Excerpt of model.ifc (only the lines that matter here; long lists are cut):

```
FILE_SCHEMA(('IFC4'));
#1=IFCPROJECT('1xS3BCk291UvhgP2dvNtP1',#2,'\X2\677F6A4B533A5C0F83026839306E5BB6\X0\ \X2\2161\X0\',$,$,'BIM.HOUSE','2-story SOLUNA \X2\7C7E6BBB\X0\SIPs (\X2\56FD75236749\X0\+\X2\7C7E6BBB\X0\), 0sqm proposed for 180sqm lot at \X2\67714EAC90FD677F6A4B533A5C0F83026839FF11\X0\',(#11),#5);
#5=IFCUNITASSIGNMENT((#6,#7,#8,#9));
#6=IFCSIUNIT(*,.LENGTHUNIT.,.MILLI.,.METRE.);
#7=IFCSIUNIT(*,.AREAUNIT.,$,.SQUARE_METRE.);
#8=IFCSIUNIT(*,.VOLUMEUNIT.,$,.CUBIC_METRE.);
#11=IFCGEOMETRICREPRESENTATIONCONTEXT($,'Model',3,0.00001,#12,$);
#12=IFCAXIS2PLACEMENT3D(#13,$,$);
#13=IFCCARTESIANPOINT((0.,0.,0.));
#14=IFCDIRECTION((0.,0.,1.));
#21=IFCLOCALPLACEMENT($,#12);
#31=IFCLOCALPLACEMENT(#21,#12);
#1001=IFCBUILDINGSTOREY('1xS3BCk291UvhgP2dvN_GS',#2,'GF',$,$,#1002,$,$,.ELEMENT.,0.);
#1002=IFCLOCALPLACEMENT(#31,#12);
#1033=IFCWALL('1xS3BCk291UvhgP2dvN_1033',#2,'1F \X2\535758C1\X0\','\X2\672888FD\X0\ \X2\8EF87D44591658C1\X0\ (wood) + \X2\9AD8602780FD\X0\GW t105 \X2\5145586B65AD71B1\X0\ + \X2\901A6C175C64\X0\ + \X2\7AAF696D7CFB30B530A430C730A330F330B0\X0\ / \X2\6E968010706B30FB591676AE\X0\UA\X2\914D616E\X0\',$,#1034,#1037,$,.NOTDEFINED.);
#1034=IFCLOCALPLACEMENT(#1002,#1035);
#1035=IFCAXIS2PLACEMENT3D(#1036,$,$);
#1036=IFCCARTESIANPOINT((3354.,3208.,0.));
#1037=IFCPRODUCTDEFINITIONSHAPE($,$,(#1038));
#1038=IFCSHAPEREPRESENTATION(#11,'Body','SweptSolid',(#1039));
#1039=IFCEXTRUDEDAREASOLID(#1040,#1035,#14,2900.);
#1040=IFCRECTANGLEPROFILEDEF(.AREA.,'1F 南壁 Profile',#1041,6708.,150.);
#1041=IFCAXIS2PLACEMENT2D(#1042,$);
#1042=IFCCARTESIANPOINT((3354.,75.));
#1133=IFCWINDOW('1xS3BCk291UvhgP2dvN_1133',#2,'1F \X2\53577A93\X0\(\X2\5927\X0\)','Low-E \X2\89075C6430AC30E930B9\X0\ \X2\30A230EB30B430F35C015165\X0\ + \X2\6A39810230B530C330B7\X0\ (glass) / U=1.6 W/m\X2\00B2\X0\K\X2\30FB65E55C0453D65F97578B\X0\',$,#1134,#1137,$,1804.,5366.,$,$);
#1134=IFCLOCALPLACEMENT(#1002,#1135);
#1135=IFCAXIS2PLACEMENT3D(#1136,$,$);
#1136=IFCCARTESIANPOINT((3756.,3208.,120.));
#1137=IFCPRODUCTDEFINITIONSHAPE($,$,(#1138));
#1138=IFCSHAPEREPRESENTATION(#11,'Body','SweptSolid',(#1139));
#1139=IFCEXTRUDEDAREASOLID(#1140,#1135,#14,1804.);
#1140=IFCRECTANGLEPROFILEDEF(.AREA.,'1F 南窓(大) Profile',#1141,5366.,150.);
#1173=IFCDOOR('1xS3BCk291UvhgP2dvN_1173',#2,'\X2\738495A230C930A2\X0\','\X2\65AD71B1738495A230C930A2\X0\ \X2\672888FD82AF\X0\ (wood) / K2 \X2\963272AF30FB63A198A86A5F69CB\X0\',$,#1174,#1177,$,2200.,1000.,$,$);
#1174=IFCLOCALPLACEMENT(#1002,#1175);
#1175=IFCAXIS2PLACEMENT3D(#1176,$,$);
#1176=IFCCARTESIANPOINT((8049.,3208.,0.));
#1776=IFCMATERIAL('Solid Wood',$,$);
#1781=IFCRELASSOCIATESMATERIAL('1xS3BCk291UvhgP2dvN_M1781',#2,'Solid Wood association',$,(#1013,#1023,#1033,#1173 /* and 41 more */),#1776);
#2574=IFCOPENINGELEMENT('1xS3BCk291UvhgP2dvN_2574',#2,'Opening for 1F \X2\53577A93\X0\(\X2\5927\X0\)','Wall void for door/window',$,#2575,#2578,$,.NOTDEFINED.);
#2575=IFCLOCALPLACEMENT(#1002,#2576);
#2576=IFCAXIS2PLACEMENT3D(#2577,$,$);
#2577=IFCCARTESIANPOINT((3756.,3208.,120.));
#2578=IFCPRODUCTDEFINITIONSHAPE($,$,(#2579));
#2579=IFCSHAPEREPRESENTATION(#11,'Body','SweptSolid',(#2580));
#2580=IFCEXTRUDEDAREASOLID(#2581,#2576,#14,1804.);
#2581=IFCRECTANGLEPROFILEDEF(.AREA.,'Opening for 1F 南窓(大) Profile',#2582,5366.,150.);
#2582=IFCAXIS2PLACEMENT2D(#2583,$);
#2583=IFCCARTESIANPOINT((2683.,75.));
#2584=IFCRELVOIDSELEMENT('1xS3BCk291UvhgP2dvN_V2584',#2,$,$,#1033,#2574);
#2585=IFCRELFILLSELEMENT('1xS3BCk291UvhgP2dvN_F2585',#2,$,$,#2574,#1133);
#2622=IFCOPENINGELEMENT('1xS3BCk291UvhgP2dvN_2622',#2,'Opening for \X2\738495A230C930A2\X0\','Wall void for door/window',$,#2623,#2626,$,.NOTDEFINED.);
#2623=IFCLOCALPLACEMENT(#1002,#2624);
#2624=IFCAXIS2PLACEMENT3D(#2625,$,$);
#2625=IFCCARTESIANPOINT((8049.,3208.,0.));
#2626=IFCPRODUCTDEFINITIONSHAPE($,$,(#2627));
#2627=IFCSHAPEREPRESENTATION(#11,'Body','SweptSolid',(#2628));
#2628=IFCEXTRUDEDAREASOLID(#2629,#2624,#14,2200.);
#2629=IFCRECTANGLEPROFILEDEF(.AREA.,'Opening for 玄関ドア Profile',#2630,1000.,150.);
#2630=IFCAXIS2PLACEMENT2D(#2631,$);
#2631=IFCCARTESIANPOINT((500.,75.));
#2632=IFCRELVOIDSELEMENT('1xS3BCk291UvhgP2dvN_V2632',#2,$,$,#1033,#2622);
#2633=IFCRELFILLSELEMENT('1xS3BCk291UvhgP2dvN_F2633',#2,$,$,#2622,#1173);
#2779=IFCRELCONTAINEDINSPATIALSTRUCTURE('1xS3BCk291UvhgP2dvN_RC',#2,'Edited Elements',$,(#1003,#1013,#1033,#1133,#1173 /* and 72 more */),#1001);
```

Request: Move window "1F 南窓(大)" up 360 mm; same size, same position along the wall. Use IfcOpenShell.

```python
import numpy as np
import ifcopenshell
import ifcopenshell.api.geometry
import ifcopenshell.util.placement
import ifcopenshell.util.unit

model = ifcopenshell.open("model.ifc")
unit_scale = ifcopenshell.util.unit.calculate_unit_scale(model)

window = model.by_guid("1xS3BCk291UvhgP2dvN_1133")
opening = window.FillsVoids[0].RelatingOpeningElement
dz = 0.36 / unit_scale

shift = np.array([0.0, 0.0, dz])
# The window is not placed relative to its opening, so move both.
for product in (opening, window):
    matrix = ifcopenshell.util.placement.get_local_placement(product.ObjectPlacement)
    matrix[:3, 3] += shift
    ifcopenshell.api.geometry.edit_object_placement(model, product=product, matrix=matrix, is_si=False)

print(f"moved by {dz * unit_scale:+.3f} m")

model.write("model_edited.ifc")
```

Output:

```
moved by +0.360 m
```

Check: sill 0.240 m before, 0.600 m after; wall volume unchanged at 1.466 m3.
